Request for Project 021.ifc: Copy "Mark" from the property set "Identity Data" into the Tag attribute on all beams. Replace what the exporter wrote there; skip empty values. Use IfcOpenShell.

First a look at what the model holds.

```python
import ifcopenshell
import ifcopenshell.util.element

model = ifcopenshell.open("Project 021.ifc")
print(model.schema)
beams = model.by_type("IfcBeam")
print(len(beams), "beams")
for e in beams[:8]:
    source = ifcopenshell.util.element.get_pset(e, "Identity Data", "Mark")
    target = e.Tag
    print(e.id(), repr(source), repr(target), sep=" | ")
```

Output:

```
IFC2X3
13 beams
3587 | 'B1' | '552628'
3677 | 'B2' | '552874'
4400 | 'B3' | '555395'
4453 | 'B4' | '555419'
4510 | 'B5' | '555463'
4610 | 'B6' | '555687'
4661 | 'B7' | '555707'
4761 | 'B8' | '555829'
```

```python
import ifcopenshell
import ifcopenshell.util.element

model = ifcopenshell.open("Project 021.ifc")

count = 0
for e in model.by_type("IfcBeam"):
    value = ifcopenshell.util.element.get_pset(e, "Identity Data", "Mark")
    current = e.Tag
    if not value or not value.strip() or current == value:
        continue
    e.Tag = value
    count += 1

print(count, "beams updated")

model.write("Project 021_edited.ifc")
```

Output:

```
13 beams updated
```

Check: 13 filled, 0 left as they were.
